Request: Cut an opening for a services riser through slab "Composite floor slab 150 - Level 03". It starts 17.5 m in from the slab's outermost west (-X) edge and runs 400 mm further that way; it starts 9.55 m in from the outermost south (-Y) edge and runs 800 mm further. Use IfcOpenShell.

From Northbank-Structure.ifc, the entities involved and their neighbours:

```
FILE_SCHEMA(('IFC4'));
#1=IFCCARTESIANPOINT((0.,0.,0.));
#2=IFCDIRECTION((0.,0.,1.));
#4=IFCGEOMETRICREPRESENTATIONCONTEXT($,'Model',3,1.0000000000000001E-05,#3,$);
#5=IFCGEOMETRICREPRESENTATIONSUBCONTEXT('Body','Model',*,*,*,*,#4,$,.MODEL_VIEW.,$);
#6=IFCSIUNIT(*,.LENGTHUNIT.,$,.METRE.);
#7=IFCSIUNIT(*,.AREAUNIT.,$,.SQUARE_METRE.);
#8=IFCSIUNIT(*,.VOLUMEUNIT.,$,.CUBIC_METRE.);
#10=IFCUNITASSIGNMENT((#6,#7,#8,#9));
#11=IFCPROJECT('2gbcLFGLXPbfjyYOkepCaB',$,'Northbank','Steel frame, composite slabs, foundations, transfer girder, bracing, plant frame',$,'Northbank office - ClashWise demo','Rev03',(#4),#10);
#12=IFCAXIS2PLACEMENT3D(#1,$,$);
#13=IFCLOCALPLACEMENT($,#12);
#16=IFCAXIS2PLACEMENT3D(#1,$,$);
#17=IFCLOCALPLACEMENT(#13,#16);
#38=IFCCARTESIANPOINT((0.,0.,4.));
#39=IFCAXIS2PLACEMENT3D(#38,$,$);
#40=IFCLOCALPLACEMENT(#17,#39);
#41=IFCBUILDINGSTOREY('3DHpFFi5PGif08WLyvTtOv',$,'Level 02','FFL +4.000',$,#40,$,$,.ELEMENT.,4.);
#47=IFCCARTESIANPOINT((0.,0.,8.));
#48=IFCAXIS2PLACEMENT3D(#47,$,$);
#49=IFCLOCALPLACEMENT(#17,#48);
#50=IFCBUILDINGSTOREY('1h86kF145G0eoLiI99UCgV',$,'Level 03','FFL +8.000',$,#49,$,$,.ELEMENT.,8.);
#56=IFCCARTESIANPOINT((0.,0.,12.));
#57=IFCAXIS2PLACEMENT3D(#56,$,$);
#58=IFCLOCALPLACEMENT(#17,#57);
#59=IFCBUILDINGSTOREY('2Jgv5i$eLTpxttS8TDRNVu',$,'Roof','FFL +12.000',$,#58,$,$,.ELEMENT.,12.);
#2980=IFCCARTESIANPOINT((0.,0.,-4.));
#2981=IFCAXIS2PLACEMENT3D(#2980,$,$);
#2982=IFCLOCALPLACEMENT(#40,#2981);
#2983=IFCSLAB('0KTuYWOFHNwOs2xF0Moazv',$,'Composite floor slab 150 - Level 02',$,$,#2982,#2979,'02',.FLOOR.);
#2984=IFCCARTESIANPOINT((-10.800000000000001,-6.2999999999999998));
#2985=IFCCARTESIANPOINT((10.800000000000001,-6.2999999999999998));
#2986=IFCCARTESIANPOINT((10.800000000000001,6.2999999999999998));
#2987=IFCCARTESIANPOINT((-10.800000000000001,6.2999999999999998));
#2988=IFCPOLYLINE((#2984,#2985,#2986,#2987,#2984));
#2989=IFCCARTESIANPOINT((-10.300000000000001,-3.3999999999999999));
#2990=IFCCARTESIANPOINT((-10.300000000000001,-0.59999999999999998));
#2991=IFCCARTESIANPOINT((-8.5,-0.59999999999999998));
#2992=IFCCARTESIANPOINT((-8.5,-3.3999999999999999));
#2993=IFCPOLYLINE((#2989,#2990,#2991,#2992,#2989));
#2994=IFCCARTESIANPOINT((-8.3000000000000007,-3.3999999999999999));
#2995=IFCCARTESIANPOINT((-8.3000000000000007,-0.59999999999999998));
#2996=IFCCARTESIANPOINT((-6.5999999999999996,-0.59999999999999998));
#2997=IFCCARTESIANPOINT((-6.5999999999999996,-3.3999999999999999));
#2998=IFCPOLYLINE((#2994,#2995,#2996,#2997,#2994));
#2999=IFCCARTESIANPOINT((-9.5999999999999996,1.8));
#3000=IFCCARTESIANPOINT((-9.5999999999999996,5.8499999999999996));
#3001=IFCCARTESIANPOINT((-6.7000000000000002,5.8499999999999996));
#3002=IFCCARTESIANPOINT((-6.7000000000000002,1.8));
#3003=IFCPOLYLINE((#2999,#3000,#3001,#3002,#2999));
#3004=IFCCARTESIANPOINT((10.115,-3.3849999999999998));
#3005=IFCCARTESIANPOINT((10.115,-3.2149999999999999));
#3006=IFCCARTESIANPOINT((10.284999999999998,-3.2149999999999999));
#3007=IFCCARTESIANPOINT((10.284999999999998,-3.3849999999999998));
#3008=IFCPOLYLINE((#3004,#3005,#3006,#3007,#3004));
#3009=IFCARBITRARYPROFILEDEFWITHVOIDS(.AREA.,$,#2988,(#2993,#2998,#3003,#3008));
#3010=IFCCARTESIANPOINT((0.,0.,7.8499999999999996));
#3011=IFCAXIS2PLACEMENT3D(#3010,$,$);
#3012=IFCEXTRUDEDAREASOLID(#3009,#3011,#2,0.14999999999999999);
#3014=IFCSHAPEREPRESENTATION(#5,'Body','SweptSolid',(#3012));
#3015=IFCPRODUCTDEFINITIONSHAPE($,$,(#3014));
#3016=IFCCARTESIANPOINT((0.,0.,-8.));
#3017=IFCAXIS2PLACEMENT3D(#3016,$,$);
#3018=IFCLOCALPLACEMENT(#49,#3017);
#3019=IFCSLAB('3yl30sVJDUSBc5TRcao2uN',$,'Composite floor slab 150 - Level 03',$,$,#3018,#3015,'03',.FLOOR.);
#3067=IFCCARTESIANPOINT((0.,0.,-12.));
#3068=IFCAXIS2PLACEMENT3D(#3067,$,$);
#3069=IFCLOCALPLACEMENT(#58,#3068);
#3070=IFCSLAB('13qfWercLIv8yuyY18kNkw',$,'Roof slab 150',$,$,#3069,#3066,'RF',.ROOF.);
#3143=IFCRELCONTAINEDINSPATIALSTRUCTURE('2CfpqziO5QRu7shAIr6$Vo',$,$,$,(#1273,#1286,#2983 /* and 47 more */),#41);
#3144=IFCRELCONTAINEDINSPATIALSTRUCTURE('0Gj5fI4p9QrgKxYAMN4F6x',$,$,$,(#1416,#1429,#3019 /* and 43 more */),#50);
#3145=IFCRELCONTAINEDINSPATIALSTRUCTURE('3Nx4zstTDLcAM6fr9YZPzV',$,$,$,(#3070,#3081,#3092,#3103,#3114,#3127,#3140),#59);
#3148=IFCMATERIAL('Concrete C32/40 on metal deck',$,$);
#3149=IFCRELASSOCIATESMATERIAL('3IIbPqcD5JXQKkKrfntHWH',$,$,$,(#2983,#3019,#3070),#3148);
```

```python
import numpy as np
import ifcopenshell
import ifcopenshell.api.feature
import ifcopenshell.api.geometry
import ifcopenshell.api.root
import ifcopenshell.geom
import ifcopenshell.util.placement
import ifcopenshell.util.representation
import ifcopenshell.util.shape
import ifcopenshell.util.unit

model = ifcopenshell.open("Northbank-Structure.ifc")
unit_scale = ifcopenshell.util.unit.calculate_unit_scale(model)
settings = ifcopenshell.geom.settings()


def volume(element):
    """Net volume in cubic metres, openings subtracted."""
    shape = ifcopenshell.geom.create_shape(settings, element)
    return ifcopenshell.util.shape.get_volume(shape.geometry)


slab = model.by_id(3019)
before = volume(slab)

# Extent in the slab's own axes, in metres. The edges named are its -X and -Y sides.
slab_shape = ifcopenshell.geom.create_shape(settings, slab)
vertices = ifcopenshell.util.shape.get_vertices(slab_shape.geometry)
x_min, y_min, bottom = vertices.min(axis=0)
top = vertices[:, 2].max()

opening = ifcopenshell.api.root.create_entity(model, ifc_class="IfcOpeningElement", name="Services riser opening", predefined_type="OPENING")
context = ifcopenshell.util.representation.get_context(model, "Model", "Body", "MODEL_VIEW")
width, depth = 0.4, 0.8
outline = [(0.0, 0.0), (width, 0.0), (width, depth), (0.0, depth), (0.0, 0.0)]
# Overshoot both faces by 50 mm so the cut is clean.
shape = ifcopenshell.api.geometry.add_slab_representation(
    model, context=context, depth=top - bottom + 0.1, polyline=outline
)
ifcopenshell.api.geometry.assign_representation(model, product=opening, representation=shape)

matrix = ifcopenshell.util.placement.get_local_placement(slab.ObjectPlacement)
matrix[:, 3] = matrix @ np.append(np.array([x_min + 17.5, y_min + 9.55, bottom - 0.05]) / unit_scale, 1.0)
ifcopenshell.api.geometry.edit_object_placement(model, product=opening, matrix=matrix, is_si=False)
ifcopenshell.api.feature.add_feature(model, feature=opening, element=slab)

after = volume(slab)

print(f"slab volume {before:.3f} -> {after:.3f} m3")

model.write("Northbank-Structure-out.ifc")
```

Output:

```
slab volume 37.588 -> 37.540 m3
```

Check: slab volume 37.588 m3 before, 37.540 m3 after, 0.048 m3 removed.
